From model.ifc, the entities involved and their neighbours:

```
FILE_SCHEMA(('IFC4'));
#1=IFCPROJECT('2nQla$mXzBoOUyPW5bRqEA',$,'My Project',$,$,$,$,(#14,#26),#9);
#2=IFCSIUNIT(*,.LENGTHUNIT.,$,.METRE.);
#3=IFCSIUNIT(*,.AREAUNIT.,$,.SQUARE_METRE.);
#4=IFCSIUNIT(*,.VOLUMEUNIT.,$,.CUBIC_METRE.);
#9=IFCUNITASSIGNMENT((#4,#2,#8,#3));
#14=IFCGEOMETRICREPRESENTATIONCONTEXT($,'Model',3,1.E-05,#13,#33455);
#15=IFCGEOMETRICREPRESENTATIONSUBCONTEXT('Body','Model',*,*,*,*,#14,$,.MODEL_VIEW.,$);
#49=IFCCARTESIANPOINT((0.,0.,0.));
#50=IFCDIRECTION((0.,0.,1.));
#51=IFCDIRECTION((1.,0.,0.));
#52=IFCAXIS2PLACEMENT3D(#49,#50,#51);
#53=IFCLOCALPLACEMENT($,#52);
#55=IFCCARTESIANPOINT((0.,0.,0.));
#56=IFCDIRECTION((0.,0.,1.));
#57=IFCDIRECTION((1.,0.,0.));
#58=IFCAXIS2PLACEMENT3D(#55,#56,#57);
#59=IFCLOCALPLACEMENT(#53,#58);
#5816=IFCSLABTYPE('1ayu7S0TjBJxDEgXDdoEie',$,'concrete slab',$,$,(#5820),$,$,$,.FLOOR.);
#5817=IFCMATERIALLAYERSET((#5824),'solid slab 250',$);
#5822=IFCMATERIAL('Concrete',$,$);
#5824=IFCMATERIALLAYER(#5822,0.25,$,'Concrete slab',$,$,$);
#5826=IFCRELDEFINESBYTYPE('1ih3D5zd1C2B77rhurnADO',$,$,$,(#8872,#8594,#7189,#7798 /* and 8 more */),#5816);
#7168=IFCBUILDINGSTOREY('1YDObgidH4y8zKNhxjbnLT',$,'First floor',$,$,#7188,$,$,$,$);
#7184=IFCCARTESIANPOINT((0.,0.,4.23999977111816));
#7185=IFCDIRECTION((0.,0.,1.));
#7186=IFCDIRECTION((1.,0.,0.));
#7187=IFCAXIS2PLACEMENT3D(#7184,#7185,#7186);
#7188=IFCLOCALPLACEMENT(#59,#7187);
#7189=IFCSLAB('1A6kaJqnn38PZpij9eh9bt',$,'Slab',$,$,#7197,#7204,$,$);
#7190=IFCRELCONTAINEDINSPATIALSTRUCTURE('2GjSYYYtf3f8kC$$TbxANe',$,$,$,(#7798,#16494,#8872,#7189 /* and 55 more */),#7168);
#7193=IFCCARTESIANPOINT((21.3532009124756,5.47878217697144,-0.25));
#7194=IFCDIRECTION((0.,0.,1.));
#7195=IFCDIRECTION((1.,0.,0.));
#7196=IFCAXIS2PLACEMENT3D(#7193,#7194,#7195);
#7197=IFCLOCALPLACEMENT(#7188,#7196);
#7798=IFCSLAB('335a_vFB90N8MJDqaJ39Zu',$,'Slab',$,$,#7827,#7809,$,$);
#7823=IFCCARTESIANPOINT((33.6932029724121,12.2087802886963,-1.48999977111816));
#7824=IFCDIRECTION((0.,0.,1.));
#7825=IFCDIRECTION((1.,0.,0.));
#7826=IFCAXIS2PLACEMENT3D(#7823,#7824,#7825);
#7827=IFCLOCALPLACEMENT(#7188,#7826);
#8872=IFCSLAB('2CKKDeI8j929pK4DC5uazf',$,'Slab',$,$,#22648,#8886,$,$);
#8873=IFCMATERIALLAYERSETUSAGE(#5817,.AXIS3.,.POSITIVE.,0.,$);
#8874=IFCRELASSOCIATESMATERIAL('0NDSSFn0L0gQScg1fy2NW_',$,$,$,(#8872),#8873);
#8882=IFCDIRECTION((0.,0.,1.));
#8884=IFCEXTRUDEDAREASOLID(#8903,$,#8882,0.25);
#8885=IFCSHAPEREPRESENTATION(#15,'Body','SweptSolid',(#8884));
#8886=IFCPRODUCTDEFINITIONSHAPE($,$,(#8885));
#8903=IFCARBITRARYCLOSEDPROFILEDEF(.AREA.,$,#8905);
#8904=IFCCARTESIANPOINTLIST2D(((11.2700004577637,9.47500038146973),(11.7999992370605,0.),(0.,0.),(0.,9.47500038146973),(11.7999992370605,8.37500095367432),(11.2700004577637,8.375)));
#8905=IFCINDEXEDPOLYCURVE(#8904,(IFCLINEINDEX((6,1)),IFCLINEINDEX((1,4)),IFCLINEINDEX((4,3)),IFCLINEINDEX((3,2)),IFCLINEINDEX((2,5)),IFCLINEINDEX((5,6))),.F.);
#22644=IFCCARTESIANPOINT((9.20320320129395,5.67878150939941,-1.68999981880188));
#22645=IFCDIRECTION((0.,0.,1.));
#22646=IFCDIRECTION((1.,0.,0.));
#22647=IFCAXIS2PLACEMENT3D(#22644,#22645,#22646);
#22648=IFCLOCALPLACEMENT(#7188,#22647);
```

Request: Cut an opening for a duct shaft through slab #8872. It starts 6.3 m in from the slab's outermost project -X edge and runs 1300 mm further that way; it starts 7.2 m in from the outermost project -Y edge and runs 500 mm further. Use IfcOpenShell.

```python
import numpy as np
import ifcopenshell
import ifcopenshell.api.feature
import ifcopenshell.api.geometry
import ifcopenshell.api.root
import ifcopenshell.geom
import ifcopenshell.util.placement
import ifcopenshell.util.representation
import ifcopenshell.util.shape
import ifcopenshell.util.unit

model = ifcopenshell.open("model.ifc")
unit_scale = ifcopenshell.util.unit.calculate_unit_scale(model)
settings = ifcopenshell.geom.settings()


def volume(element):
    """Net volume in cubic metres, openings subtracted."""
    shape = ifcopenshell.geom.create_shape(settings, element)
    return ifcopenshell.util.shape.get_volume(shape.geometry)


slab = model.by_id(8872)
before = volume(slab)

# Extent in the slab's own axes, in metres. The edges named are its -X and -Y sides.
slab_shape = ifcopenshell.geom.create_shape(settings, slab)
vertices = ifcopenshell.util.shape.get_vertices(slab_shape.geometry)
x_min, y_min, bottom = vertices.min(axis=0)
top = vertices[:, 2].max()

opening = ifcopenshell.api.root.create_entity(model, ifc_class="IfcOpeningElement", name="Duct shaft opening", predefined_type="OPENING")
context = ifcopenshell.util.representation.get_context(model, "Model", "Body", "MODEL_VIEW")
width, depth = 1.3, 0.5
outline = [(0.0, 0.0), (width, 0.0), (width, depth), (0.0, depth), (0.0, 0.0)]
# Overshoot both faces by 50 mm so the cut is clean.
shape = ifcopenshell.api.geometry.add_slab_representation(
    model, context=context, depth=top - bottom + 0.1, polyline=outline
)
ifcopenshell.api.geometry.assign_representation(model, product=opening, representation=shape)

matrix = ifcopenshell.util.placement.get_local_placement(slab.ObjectPlacement)
matrix[:, 3] = matrix @ np.append(np.array([x_min + 6.3, y_min + 7.2, bottom - 0.05]) / unit_scale, 1.0)
ifcopenshell.api.geometry.edit_object_placement(model, product=opening, matrix=matrix, is_si=False)
ifcopenshell.api.feature.add_feature(model, feature=opening, element=slab)

after = volume(slab)

print(f"slab volume {before:.3f} -> {after:.3f} m3")

model.write("model_v2.ifc")
```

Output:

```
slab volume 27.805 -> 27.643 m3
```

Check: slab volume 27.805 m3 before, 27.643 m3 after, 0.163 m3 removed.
